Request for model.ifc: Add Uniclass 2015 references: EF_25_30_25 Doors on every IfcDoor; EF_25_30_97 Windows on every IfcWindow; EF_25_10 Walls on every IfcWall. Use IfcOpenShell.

First a look at what the model holds.

```python
import ifcopenshell

model = ifcopenshell.open("model.ifc")
print(model.schema)
print("classifications:", [c.Name for c in model.by_type("IfcClassification")])
for ifc_class in ("IfcDoor", "IfcRoof", "IfcStair", "IfcWall", "IfcWindow"):
    print(ifc_class, len(model.by_type(ifc_class)))
```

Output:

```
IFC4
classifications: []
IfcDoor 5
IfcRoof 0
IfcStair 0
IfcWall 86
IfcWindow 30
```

```python
import ifcopenshell
import ifcopenshell.api.classification

model = ifcopenshell.open("model.ifc")

system = ifcopenshell.api.classification.add_classification(model, classification="Uniclass 2015")

codes = {
    "IfcDoor": ("EF_25_30_25", "Doors"),
    "IfcWindow": ("EF_25_30_97", "Windows"),
    "IfcWall": ("EF_25_10", "Walls"),
}
for ifc_class, (code, name) in codes.items():
    products = model.by_type(ifc_class)
    ifcopenshell.api.classification.add_reference(
        model, products=products, classification=system, identification=code, name=name
    )
    print(code, len(products))

model.write("model_edited.ifc")
```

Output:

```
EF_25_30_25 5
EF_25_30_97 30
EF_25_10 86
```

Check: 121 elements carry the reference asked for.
